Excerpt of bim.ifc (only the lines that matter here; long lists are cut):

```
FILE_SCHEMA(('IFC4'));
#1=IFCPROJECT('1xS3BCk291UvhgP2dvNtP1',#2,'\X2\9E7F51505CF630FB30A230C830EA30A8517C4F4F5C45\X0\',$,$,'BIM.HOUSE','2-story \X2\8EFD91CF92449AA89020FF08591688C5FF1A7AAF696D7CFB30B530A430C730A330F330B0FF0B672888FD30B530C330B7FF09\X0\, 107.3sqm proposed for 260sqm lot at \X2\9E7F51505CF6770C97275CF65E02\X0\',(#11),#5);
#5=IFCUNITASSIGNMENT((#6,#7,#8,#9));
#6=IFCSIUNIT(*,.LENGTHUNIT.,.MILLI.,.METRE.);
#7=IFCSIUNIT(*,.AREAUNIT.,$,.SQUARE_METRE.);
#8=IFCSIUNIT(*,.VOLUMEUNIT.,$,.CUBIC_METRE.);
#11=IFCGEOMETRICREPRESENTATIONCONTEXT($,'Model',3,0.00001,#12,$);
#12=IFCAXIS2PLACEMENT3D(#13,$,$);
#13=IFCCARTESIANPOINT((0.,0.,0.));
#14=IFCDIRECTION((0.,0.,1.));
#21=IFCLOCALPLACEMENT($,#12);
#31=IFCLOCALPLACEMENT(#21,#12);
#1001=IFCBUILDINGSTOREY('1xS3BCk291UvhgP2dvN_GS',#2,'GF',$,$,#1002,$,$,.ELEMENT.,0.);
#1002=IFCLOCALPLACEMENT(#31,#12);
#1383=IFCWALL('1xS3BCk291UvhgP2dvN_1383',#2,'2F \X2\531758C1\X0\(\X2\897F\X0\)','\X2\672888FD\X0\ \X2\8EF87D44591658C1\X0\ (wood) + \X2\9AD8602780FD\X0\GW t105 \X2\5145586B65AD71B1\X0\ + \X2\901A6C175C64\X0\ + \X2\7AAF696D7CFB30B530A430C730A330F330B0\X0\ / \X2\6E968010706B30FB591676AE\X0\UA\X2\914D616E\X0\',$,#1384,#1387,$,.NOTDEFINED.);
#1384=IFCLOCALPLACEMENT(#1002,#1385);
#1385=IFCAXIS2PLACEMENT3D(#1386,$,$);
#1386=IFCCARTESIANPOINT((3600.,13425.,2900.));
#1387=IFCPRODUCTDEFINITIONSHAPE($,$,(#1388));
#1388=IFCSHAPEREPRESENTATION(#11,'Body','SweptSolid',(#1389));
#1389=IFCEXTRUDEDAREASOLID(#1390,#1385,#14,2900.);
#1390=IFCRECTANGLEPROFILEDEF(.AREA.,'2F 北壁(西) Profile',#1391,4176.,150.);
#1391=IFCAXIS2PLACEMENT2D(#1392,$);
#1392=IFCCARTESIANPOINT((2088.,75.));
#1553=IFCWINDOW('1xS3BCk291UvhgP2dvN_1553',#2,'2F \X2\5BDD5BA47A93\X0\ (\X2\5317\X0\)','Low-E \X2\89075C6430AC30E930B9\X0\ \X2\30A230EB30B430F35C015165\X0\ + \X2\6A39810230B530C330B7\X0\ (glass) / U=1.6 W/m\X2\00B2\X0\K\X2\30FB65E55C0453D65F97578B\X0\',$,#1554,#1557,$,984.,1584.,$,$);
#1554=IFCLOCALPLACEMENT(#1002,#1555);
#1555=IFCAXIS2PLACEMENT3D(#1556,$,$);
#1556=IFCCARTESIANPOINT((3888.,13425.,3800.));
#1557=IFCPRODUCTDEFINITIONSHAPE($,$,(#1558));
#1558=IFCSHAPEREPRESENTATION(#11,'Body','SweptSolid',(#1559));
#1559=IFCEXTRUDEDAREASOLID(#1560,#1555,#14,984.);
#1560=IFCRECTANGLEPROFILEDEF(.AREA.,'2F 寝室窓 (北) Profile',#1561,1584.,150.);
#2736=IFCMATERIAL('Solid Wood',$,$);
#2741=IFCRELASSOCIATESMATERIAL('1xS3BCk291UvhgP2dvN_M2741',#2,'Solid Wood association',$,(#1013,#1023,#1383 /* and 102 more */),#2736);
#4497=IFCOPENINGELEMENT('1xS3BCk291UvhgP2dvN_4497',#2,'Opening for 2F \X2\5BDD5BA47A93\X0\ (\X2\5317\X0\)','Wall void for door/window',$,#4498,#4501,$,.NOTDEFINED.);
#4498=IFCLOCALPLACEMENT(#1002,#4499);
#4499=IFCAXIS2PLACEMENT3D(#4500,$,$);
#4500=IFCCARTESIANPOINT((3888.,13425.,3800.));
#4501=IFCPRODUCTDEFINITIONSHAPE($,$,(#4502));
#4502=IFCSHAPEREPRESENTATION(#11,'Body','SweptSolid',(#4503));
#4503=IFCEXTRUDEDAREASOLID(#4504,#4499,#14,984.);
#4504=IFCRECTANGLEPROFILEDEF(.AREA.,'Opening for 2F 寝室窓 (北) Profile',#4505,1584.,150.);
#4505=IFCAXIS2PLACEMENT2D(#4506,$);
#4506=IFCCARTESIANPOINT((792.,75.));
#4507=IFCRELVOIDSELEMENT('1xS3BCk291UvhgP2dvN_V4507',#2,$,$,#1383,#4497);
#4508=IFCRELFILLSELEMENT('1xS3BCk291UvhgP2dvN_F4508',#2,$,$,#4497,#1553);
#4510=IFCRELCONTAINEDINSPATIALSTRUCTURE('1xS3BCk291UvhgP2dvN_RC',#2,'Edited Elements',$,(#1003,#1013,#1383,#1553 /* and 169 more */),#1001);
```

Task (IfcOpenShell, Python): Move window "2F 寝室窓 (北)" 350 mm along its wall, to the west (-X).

```python
import ifcopenshell
import ifcopenshell.api.geometry
import ifcopenshell.util.placement

model = ifcopenshell.open("bim.ifc")

window = model.by_guid("1xS3BCk291UvhgP2dvN_1553")
opening = window.FillsVoids[0].RelatingOpeningElement
wall = opening.VoidsElements[0].RelatingBuildingElement

wall_matrix = ifcopenshell.util.placement.get_local_placement(wall.ObjectPlacement)
shift = wall_matrix[:3, 0] * -350.0
before = ifcopenshell.util.placement.get_local_placement(window.ObjectPlacement)[:3, 3].copy()

# The window is not placed relative to its opening, so move both.
for product in (opening, window):
    matrix = ifcopenshell.util.placement.get_local_placement(product.ObjectPlacement)
    matrix[:3, 3] += shift
    ifcopenshell.api.geometry.edit_object_placement(model, product=product, matrix=matrix, is_si=False)

after = ifcopenshell.util.placement.get_local_placement(window.ObjectPlacement)[:3, 3]
print("window moved by", (after - before).round(3) + 0.0)

model.write("bim_rev.ifc")
```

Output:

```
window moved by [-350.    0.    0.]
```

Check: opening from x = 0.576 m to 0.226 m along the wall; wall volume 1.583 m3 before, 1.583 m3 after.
